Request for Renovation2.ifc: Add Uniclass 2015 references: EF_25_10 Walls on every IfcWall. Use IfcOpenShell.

First a look at what the model holds.

```python
import ifcopenshell

model = ifcopenshell.open("Renovation2.ifc")
print(model.schema)
print("classifications:", [c.Name for c in model.by_type("IfcClassification")])
for ifc_class in ("IfcDoor", "IfcRoof", "IfcStair", "IfcWall", "IfcWindow"):
    print(ifc_class, len(model.by_type(ifc_class)))
```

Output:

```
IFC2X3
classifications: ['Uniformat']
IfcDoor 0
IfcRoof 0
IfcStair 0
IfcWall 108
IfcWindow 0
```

```python
import ifcopenshell
import ifcopenshell.api.classification

model = ifcopenshell.open("Renovation2.ifc")

# IFC2X3 requires Source and Edition and has no link from the project to the system.
system = model.create_entity("IfcClassification", Source="NBS", Edition="2015", Name="Uniclass 2015")

codes = {
    "IfcWall": ("EF_25_10", "Walls"),
}
for ifc_class, (code, name) in codes.items():
    products = model.by_type(ifc_class)
    ifcopenshell.api.classification.add_reference(
        model, products=products, classification=system, identification=code, name=name
    )
    print(code, len(products))

model.write("Renovation2_v2.ifc")
```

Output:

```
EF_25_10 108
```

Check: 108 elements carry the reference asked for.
